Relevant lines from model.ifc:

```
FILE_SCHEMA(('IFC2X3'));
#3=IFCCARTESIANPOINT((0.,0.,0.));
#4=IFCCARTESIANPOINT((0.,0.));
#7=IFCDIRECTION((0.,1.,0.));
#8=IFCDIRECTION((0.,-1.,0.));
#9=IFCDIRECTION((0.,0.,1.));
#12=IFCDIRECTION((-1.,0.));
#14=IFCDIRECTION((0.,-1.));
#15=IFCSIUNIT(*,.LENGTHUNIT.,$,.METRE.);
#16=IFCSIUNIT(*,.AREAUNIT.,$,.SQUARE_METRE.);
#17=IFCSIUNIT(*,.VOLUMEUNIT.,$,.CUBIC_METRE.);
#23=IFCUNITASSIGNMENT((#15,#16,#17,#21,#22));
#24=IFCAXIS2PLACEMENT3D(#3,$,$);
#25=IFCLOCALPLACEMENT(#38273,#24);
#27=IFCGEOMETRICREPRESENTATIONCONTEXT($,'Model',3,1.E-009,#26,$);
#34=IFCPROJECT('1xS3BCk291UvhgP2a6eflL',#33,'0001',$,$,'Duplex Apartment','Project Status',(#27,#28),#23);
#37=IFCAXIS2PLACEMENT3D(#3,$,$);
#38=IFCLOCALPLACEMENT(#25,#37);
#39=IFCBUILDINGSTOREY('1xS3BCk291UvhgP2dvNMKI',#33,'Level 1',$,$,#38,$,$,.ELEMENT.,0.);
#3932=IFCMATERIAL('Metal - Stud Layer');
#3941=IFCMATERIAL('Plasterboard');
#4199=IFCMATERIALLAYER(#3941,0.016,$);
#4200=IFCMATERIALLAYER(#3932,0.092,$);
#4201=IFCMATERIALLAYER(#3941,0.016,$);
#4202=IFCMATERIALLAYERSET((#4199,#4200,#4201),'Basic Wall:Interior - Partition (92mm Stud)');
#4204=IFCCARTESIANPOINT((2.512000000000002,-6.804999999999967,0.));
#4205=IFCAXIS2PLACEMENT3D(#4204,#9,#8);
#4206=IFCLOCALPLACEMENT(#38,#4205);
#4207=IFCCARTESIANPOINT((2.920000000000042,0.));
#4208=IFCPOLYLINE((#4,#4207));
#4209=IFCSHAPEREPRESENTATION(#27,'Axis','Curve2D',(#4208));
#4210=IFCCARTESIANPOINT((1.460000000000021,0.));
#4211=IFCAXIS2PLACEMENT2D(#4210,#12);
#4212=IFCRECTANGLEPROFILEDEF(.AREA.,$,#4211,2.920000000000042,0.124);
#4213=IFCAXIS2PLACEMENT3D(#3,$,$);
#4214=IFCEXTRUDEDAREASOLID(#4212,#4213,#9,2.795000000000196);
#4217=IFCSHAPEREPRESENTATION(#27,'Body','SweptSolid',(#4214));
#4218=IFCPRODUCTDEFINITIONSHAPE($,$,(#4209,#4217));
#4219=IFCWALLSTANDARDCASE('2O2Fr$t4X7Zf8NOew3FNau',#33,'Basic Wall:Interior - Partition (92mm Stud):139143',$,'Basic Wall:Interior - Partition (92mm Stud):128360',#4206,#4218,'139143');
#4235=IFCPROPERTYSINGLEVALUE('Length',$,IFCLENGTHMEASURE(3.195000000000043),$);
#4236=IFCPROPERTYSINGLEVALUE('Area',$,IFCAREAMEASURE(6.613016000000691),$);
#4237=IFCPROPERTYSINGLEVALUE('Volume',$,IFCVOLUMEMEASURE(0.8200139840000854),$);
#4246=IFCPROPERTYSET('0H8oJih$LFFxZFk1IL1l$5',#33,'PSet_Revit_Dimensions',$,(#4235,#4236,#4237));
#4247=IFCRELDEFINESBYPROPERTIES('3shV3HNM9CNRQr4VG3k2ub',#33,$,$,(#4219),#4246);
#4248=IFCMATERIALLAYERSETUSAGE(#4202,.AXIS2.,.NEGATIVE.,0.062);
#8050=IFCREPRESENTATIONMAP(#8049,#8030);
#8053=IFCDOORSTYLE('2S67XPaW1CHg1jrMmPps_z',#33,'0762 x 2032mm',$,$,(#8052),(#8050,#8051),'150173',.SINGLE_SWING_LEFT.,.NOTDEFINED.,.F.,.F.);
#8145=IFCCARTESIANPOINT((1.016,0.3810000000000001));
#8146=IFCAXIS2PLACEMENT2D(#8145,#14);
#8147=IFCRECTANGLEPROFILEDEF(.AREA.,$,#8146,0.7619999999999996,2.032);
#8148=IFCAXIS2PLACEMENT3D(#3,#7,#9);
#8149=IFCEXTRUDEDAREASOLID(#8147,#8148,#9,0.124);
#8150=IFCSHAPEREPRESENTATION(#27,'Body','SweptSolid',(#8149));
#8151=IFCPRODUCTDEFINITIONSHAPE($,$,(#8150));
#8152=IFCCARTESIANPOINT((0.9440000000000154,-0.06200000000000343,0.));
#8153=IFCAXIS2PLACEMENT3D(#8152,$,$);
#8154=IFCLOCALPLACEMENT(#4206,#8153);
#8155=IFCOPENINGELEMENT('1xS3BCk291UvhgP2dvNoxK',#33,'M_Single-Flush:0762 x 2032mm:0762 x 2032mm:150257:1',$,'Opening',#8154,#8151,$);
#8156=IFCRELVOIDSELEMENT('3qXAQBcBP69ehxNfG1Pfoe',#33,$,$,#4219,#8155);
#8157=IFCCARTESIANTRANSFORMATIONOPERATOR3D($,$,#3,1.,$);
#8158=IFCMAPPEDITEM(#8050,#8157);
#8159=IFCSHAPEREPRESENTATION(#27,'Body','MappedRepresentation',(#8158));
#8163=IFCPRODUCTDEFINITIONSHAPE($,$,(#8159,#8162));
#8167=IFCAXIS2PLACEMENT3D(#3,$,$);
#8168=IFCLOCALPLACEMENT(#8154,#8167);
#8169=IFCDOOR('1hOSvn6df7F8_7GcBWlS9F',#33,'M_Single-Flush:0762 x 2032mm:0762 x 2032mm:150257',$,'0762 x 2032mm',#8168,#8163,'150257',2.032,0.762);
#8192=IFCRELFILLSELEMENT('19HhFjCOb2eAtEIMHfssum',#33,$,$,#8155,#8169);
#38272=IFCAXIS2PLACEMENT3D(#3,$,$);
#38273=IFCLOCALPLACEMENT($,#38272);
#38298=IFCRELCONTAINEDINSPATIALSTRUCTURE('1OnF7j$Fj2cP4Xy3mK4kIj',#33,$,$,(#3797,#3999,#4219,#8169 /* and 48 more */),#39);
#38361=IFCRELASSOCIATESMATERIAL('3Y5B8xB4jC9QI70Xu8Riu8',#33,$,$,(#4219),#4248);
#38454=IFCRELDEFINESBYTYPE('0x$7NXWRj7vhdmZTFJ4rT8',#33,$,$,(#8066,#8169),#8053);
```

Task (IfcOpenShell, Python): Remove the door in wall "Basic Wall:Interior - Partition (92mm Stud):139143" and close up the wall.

```python
import ifcopenshell
import ifcopenshell.api.feature
import ifcopenshell.api.pset
import ifcopenshell.api.root
import ifcopenshell.geom
import ifcopenshell.util.element
import ifcopenshell.util.shape
import ifcopenshell.util.unit

model = ifcopenshell.open("model.ifc")
area_scale = ifcopenshell.util.unit.calculate_unit_scale(model, "AREAUNIT")
volume_scale = ifcopenshell.util.unit.calculate_unit_scale(model, "VOLUMEUNIT")
settings = ifcopenshell.geom.settings()


def volume(element):
    """Net volume in cubic metres, openings subtracted."""
    shape = ifcopenshell.geom.create_shape(settings, element)
    return ifcopenshell.util.shape.get_volume(shape.geometry)


door = model.by_id(8169)
opening = door.FillsVoids[0].RelatingOpeningElement
wall = opening.VoidsElements[0].RelatingBuildingElement
before = volume(wall)

ifcopenshell.api.root.remove_product(model, product=door)
ifcopenshell.api.feature.remove_feature(model, feature=opening)

after = volume(wall)
thickness = 0.124  # wall thickness in metres

# Update the wall's stored quantities.
pset = model.by_id(ifcopenshell.util.element.get_pset(wall, "PSet_Revit_Dimensions", should_inherit=False)["id"])
ifcopenshell.api.pset.edit_pset(model, pset=pset, properties={
    "Area": model.create_entity("IfcAreaMeasure", after / thickness / area_scale),
    "Volume": model.create_entity("IfcVolumeMeasure", after / volume_scale),
})

print(f"wall volume {before:.3f} -> {after:.3f} m3")

model.write("model_updated.ifc")
```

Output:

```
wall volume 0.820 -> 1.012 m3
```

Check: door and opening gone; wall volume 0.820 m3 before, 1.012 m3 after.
